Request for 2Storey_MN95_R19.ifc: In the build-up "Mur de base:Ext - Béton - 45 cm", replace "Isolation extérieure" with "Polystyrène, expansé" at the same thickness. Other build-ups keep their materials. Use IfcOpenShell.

First a look at what the model holds.

```python
import ifcopenshell
import ifcopenshell.util.element

model = ifcopenshell.open("2Storey_MN95_R19.ifc")
print(model.schema)
for layer_set in model.by_type("IfcMaterialLayerSet"):
    if layer_set.LayerSetName == "Mur de base:Ext - Béton - 45 cm":
        for layer in layer_set.MaterialLayers:
            print(layer.id(), layer.Material and layer.Material.Name, layer.LayerThickness, sep=" | ")
        print(len(ifcopenshell.util.element.get_elements_by_material(model, layer_set)), "elements and types use it")
print(sorted(m.Name for m in model.by_type("IfcMaterial") if m.Name)[:60])
```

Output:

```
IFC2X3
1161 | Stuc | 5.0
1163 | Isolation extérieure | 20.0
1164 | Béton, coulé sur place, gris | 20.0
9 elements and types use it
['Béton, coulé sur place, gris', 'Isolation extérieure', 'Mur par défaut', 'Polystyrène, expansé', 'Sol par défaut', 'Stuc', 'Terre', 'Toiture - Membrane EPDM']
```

```python
import ifcopenshell
import ifcopenshell.api.material

model = ifcopenshell.open("2Storey_MN95_R19.ifc")

layer_set = next(s for s in model.by_type("IfcMaterialLayerSet") if s.LayerSetName == "Mur de base:Ext - Béton - 45 cm")
layer = next(l for l in layer_set.MaterialLayers if l.Material and l.Material.Name == "Isolation extérieure")
material = next(m for m in model.by_type("IfcMaterial") if m.Name == "Polystyrène, expansé")

# Point this one layer at the other material; renaming the old one would change it everywhere.
ifcopenshell.api.material.edit_layer(model, layer=layer, attributes={}, material=material)

print([l.Material.Name if l.Material else None for l in layer_set.MaterialLayers])

model.write("2Storey_MN95_R19_v2.ifc")
```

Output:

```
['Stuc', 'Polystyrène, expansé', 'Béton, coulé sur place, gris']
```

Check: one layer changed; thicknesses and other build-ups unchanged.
